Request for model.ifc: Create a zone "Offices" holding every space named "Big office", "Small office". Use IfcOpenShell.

First a look at what the model holds.

```python
import ifcopenshell

model = ifcopenshell.open("model.ifc")
print(model.schema)
seen = {}
for space in model.by_type("IfcSpace"):
    seen[space.LongName] = seen.get(space.LongName, 0) + 1
for name, count in sorted(seen.items(), key=str):
    print(count, "x", name)
print("zones:", [z.Name for z in model.by_type("IfcZone")][:20])
```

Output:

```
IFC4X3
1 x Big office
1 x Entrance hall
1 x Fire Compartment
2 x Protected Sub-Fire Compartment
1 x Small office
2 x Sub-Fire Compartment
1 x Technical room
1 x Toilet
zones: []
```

```python
import ifcopenshell
import ifcopenshell.api.group
import ifcopenshell.api.root

model = ifcopenshell.open("model.ifc")

names = {"Big office", "Small office"}
spaces = [s for s in model.by_type("IfcSpace") if s.LongName in names]

zone = ifcopenshell.api.root.create_entity(model, ifc_class="IfcZone", name="Offices")
ifcopenshell.api.group.assign_group(model, products=spaces, group=zone)
print(len(spaces), "spaces in", zone.Name)

model.write("model-out.ifc")
```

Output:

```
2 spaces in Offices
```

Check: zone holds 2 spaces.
